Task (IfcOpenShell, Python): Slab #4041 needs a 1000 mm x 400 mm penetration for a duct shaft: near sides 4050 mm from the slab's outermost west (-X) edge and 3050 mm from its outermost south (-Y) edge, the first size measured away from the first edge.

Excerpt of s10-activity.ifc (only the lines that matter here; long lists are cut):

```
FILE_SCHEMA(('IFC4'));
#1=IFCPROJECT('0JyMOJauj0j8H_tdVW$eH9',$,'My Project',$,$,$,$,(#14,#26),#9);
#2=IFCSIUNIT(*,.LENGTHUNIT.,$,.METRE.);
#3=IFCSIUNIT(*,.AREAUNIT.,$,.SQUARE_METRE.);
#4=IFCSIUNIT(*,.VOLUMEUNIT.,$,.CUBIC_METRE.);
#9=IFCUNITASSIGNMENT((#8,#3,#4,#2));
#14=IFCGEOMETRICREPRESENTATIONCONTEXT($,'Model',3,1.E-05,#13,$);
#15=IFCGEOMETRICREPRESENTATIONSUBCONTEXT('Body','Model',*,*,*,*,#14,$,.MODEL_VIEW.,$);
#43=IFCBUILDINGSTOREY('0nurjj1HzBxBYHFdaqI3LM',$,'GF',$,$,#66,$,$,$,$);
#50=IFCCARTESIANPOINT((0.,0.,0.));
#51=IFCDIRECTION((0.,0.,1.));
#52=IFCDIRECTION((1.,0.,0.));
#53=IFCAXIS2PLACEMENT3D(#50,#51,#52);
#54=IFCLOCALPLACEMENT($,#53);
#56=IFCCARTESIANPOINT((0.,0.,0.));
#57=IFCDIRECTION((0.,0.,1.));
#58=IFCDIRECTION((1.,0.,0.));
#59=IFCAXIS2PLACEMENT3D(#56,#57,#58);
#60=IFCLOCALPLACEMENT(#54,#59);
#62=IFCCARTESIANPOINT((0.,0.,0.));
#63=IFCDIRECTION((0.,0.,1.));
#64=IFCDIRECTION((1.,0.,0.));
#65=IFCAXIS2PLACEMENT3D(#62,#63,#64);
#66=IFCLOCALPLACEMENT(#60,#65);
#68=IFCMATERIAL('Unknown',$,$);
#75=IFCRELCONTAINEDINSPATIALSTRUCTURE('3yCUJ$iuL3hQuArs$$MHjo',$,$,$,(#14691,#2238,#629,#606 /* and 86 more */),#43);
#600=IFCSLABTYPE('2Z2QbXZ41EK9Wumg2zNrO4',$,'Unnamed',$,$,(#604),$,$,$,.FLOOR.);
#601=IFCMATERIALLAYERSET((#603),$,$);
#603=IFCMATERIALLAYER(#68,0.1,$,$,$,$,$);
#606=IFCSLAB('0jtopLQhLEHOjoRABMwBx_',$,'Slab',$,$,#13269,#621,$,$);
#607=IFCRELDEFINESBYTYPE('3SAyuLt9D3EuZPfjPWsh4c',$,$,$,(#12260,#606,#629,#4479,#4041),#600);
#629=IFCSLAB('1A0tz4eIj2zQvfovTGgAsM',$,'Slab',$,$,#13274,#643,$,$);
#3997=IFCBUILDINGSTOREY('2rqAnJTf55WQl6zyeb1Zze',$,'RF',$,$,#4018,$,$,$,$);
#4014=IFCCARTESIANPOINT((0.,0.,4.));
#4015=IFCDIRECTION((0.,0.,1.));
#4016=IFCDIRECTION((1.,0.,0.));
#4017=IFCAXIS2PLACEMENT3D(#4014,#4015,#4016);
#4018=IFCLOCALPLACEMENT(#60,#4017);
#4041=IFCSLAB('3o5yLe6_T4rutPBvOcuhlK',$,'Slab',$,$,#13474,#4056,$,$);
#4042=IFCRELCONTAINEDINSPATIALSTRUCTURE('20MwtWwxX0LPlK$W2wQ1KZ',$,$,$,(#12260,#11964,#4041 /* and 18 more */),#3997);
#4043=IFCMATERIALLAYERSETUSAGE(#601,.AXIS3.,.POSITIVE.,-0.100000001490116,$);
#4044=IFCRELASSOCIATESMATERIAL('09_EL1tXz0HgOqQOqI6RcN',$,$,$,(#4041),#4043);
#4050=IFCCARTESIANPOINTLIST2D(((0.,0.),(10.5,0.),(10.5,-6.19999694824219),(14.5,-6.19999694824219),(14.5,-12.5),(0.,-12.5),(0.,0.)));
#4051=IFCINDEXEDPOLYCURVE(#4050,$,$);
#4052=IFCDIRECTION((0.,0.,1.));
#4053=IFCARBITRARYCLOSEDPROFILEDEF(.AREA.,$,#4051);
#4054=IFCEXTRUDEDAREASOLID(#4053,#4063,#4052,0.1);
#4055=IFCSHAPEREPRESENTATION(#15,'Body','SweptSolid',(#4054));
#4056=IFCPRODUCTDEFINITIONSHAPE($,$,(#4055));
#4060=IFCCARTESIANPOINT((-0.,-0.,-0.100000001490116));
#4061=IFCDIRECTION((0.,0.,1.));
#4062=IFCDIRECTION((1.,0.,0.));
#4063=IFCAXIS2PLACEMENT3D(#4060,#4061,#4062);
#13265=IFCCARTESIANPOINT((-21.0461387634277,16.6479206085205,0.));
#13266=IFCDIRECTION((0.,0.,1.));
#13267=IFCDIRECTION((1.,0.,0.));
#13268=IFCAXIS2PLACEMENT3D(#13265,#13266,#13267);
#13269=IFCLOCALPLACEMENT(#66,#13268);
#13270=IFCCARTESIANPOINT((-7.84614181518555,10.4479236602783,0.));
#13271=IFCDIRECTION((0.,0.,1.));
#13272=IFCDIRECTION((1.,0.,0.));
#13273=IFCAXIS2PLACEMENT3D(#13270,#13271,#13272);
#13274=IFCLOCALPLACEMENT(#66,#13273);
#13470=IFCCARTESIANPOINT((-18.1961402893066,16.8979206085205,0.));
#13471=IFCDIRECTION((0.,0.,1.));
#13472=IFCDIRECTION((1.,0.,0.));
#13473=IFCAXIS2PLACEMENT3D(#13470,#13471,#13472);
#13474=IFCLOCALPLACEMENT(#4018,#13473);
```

```python
import numpy as np
import ifcopenshell
import ifcopenshell.api.feature
import ifcopenshell.api.geometry
import ifcopenshell.api.root
import ifcopenshell.geom
import ifcopenshell.util.placement
import ifcopenshell.util.representation
import ifcopenshell.util.shape
import ifcopenshell.util.unit

model = ifcopenshell.open("s10-activity.ifc")
unit_scale = ifcopenshell.util.unit.calculate_unit_scale(model)
settings = ifcopenshell.geom.settings()


def volume(element):
    """Net volume in cubic metres, openings subtracted."""
    shape = ifcopenshell.geom.create_shape(settings, element)
    return ifcopenshell.util.shape.get_volume(shape.geometry)


slab = model.by_guid("3o5yLe6_T4rutPBvOcuhlK")
before = volume(slab)

# Extent in the slab's own axes, in metres. The edges named are its -X and -Y sides.
slab_shape = ifcopenshell.geom.create_shape(settings, slab)
vertices = ifcopenshell.util.shape.get_vertices(slab_shape.geometry)
x_min, y_min, bottom = vertices.min(axis=0)
top = vertices[:, 2].max()

opening = ifcopenshell.api.root.create_entity(model, ifc_class="IfcOpeningElement", name="Duct shaft opening", predefined_type="OPENING")
context = ifcopenshell.util.representation.get_context(model, "Model", "Body", "MODEL_VIEW")
width, depth = 1, 0.4
outline = [(0.0, 0.0), (width, 0.0), (width, depth), (0.0, depth), (0.0, 0.0)]
# Overshoot both faces by 50 mm so the cut is clean.
shape = ifcopenshell.api.geometry.add_slab_representation(
    model, context=context, depth=top - bottom + 0.1, polyline=outline
)
ifcopenshell.api.geometry.assign_representation(model, product=opening, representation=shape)

matrix = ifcopenshell.util.placement.get_local_placement(slab.ObjectPlacement)
matrix[:, 3] = matrix @ np.append(np.array([x_min + 4.05, y_min + 3.05, bottom - 0.05]) / unit_scale, 1.0)
ifcopenshell.api.geometry.edit_object_placement(model, product=opening, matrix=matrix, is_si=False)
ifcopenshell.api.feature.add_feature(model, feature=opening, element=slab)

after = volume(slab)

print(f"slab volume {before:.3f} -> {after:.3f} m3")

model.write("s10-activity_v2.ifc")
```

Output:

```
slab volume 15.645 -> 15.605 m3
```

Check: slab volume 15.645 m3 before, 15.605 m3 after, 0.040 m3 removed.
